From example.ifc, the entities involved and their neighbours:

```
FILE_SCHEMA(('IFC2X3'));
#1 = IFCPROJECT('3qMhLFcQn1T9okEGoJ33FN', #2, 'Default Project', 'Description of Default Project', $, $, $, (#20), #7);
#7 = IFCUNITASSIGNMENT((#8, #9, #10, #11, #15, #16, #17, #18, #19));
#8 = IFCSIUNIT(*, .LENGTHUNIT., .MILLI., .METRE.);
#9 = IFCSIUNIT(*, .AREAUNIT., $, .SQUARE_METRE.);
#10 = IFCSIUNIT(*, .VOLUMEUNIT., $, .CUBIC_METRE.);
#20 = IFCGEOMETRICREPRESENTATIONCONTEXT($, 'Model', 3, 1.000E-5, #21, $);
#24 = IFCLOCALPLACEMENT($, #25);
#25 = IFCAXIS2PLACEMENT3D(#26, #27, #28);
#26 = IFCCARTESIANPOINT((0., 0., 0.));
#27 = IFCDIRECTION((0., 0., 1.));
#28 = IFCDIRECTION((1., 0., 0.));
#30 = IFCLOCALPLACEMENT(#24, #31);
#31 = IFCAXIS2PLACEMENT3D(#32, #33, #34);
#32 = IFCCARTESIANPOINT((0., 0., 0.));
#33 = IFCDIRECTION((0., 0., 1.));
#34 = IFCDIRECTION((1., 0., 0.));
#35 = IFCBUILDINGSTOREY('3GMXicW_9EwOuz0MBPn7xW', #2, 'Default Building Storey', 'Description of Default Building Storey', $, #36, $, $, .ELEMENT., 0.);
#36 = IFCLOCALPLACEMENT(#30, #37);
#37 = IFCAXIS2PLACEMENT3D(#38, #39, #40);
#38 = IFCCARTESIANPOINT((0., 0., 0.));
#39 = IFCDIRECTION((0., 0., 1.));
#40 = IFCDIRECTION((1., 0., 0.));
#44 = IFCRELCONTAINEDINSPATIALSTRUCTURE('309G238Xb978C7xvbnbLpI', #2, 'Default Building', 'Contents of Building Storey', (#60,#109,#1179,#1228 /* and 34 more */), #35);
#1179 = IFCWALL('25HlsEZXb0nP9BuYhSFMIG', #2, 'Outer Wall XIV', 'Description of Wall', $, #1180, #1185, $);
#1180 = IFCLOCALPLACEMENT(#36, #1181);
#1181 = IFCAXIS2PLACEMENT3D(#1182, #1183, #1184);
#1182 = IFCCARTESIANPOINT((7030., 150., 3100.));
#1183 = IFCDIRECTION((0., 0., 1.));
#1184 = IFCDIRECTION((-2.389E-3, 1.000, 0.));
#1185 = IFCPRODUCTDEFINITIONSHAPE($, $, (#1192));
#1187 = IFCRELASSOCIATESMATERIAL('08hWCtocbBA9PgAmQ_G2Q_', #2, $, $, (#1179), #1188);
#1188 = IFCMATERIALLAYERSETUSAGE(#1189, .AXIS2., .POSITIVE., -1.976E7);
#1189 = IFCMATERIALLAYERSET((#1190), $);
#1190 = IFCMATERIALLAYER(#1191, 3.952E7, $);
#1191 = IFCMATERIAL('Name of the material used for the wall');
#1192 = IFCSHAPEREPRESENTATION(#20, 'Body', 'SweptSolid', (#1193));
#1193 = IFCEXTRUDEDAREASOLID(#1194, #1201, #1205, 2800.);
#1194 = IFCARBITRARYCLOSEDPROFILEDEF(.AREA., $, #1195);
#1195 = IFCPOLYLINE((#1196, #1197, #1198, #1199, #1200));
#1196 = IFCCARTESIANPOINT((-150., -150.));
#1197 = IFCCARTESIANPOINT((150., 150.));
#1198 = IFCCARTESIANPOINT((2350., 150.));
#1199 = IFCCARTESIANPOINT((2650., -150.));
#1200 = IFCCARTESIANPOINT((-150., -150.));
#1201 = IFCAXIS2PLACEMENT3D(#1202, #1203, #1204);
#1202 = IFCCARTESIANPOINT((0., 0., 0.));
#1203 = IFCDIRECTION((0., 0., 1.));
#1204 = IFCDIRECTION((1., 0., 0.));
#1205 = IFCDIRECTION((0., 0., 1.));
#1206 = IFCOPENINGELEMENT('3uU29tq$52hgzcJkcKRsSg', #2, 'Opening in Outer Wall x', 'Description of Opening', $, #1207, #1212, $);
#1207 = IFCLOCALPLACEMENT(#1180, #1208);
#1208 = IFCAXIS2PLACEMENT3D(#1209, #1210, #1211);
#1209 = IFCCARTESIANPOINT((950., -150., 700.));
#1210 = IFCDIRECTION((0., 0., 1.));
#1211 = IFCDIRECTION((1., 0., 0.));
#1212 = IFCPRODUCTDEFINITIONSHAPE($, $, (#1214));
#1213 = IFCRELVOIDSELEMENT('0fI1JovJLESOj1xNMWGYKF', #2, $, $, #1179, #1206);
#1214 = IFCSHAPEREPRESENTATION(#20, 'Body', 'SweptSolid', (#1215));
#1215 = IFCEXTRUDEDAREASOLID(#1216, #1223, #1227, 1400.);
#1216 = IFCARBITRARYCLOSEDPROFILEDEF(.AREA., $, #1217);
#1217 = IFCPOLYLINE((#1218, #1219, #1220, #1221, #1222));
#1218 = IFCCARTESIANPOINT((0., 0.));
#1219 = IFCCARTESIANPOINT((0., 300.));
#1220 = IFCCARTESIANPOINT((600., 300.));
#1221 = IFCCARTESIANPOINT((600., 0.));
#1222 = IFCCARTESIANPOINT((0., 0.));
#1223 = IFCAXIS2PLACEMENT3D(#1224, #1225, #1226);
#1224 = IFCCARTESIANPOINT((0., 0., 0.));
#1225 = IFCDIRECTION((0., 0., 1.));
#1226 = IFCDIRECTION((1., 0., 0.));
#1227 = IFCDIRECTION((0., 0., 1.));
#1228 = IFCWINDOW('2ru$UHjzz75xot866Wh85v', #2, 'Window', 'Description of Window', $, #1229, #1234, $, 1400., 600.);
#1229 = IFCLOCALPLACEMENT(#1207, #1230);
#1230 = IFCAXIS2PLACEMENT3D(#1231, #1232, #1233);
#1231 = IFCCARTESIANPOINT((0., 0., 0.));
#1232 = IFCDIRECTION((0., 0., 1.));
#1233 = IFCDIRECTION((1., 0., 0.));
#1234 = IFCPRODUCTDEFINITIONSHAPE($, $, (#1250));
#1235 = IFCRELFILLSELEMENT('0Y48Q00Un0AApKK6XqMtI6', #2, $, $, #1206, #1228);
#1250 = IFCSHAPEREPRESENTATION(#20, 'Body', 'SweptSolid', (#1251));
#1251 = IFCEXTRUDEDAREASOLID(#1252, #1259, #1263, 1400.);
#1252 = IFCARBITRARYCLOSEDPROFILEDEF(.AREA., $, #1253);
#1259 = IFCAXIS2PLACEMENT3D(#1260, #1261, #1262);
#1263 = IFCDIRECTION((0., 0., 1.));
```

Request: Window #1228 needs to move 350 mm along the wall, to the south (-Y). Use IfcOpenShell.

```python
import ifcopenshell
import ifcopenshell.api.geometry
import ifcopenshell.util.placement
import ifcopenshell.util.unit

model = ifcopenshell.open("example.ifc")
unit_scale = ifcopenshell.util.unit.calculate_unit_scale(model)

window = model.by_id(1228)
opening = window.FillsVoids[0].RelatingOpeningElement
wall = opening.VoidsElements[0].RelatingBuildingElement

wall_matrix = ifcopenshell.util.placement.get_local_placement(wall.ObjectPlacement)
shift = wall_matrix[:3, 0] * -0.35 / unit_scale
before = ifcopenshell.util.placement.get_local_placement(window.ObjectPlacement)[:3, 3].copy()

# The window is placed relative to its opening, so it follows when the opening moves.
matrix = ifcopenshell.util.placement.get_local_placement(opening.ObjectPlacement)
matrix[:3, 3] += shift
ifcopenshell.api.geometry.edit_object_placement(
    model, product=opening, matrix=matrix, is_si=False, should_transform_children=True
)

after = ifcopenshell.util.placement.get_local_placement(window.ObjectPlacement)[:3, 3]
print("window moved by", (after - before).round(3) + 0.0)

model.write("example_edited.ifc")
```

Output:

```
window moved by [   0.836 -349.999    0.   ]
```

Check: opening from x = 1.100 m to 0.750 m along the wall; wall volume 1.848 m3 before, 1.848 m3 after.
